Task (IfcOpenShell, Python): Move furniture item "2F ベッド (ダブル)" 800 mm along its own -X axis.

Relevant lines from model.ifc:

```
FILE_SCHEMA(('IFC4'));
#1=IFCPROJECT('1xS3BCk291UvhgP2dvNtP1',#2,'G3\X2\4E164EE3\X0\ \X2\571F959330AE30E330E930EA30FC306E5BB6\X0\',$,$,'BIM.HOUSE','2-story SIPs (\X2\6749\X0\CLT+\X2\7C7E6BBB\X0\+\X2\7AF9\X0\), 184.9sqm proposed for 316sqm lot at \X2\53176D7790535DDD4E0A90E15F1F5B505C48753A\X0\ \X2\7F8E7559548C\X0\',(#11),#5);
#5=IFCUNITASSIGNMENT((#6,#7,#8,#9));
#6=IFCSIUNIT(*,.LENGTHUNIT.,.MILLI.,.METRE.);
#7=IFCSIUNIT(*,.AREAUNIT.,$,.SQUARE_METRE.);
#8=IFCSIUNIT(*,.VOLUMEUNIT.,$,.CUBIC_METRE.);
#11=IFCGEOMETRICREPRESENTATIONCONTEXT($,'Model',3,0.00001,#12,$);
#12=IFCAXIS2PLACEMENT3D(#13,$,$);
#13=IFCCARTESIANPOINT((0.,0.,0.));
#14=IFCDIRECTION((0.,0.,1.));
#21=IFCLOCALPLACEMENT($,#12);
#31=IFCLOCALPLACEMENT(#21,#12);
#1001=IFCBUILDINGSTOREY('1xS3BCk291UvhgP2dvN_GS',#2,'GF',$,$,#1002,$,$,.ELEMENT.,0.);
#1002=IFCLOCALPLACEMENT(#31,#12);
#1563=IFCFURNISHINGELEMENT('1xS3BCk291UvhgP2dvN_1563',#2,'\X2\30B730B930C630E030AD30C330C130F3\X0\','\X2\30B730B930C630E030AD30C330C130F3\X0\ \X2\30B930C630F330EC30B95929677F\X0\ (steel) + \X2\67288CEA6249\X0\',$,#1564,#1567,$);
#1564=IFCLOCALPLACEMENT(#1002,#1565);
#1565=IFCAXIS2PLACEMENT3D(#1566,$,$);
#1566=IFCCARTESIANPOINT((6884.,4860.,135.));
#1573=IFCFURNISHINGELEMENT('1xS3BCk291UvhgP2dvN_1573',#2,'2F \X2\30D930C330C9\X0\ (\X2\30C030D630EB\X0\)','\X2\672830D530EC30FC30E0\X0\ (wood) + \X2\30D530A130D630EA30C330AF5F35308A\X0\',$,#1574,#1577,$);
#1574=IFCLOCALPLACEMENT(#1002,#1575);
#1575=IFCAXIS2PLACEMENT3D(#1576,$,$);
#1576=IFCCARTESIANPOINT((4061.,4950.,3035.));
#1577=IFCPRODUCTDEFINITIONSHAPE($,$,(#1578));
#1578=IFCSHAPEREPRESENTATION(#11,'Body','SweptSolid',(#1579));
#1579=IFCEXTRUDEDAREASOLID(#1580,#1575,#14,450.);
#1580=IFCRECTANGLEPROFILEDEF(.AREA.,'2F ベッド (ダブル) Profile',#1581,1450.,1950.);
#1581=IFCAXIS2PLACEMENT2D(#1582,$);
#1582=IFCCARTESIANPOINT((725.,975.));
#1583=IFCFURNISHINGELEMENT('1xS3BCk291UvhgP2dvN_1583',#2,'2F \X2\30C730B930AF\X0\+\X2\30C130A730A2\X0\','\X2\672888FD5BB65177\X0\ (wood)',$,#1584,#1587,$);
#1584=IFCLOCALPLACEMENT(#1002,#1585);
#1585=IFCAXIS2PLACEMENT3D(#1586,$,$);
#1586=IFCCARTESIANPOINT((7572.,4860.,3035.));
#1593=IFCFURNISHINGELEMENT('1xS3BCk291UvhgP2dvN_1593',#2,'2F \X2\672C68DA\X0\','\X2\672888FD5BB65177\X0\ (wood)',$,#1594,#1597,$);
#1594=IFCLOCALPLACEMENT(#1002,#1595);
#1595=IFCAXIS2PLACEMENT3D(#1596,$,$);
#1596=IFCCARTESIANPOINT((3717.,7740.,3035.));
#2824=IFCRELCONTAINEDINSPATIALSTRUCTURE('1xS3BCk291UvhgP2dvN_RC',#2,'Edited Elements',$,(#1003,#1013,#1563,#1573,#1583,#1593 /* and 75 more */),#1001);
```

```python
import ifcopenshell
import ifcopenshell.api.geometry
import ifcopenshell.util.placement
import ifcopenshell.util.unit

model = ifcopenshell.open("model.ifc")
unit_scale = ifcopenshell.util.unit.calculate_unit_scale(model)

item = model.by_guid("1xS3BCk291UvhgP2dvN_1573")
matrix = ifcopenshell.util.placement.get_local_placement(item.ObjectPlacement)
matrix[:3, 3] -= matrix[:3, 0] * 0.8 / unit_scale
ifcopenshell.api.geometry.edit_object_placement(model, product=item, matrix=matrix, is_si=False)

print(ifcopenshell.util.placement.get_local_placement(item.ObjectPlacement).round(3) + 0.0)

model.write("model-out.ifc")
```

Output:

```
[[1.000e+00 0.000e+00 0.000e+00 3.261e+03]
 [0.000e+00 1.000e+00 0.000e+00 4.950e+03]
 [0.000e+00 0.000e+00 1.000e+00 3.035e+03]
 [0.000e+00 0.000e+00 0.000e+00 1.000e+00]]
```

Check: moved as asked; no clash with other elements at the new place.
